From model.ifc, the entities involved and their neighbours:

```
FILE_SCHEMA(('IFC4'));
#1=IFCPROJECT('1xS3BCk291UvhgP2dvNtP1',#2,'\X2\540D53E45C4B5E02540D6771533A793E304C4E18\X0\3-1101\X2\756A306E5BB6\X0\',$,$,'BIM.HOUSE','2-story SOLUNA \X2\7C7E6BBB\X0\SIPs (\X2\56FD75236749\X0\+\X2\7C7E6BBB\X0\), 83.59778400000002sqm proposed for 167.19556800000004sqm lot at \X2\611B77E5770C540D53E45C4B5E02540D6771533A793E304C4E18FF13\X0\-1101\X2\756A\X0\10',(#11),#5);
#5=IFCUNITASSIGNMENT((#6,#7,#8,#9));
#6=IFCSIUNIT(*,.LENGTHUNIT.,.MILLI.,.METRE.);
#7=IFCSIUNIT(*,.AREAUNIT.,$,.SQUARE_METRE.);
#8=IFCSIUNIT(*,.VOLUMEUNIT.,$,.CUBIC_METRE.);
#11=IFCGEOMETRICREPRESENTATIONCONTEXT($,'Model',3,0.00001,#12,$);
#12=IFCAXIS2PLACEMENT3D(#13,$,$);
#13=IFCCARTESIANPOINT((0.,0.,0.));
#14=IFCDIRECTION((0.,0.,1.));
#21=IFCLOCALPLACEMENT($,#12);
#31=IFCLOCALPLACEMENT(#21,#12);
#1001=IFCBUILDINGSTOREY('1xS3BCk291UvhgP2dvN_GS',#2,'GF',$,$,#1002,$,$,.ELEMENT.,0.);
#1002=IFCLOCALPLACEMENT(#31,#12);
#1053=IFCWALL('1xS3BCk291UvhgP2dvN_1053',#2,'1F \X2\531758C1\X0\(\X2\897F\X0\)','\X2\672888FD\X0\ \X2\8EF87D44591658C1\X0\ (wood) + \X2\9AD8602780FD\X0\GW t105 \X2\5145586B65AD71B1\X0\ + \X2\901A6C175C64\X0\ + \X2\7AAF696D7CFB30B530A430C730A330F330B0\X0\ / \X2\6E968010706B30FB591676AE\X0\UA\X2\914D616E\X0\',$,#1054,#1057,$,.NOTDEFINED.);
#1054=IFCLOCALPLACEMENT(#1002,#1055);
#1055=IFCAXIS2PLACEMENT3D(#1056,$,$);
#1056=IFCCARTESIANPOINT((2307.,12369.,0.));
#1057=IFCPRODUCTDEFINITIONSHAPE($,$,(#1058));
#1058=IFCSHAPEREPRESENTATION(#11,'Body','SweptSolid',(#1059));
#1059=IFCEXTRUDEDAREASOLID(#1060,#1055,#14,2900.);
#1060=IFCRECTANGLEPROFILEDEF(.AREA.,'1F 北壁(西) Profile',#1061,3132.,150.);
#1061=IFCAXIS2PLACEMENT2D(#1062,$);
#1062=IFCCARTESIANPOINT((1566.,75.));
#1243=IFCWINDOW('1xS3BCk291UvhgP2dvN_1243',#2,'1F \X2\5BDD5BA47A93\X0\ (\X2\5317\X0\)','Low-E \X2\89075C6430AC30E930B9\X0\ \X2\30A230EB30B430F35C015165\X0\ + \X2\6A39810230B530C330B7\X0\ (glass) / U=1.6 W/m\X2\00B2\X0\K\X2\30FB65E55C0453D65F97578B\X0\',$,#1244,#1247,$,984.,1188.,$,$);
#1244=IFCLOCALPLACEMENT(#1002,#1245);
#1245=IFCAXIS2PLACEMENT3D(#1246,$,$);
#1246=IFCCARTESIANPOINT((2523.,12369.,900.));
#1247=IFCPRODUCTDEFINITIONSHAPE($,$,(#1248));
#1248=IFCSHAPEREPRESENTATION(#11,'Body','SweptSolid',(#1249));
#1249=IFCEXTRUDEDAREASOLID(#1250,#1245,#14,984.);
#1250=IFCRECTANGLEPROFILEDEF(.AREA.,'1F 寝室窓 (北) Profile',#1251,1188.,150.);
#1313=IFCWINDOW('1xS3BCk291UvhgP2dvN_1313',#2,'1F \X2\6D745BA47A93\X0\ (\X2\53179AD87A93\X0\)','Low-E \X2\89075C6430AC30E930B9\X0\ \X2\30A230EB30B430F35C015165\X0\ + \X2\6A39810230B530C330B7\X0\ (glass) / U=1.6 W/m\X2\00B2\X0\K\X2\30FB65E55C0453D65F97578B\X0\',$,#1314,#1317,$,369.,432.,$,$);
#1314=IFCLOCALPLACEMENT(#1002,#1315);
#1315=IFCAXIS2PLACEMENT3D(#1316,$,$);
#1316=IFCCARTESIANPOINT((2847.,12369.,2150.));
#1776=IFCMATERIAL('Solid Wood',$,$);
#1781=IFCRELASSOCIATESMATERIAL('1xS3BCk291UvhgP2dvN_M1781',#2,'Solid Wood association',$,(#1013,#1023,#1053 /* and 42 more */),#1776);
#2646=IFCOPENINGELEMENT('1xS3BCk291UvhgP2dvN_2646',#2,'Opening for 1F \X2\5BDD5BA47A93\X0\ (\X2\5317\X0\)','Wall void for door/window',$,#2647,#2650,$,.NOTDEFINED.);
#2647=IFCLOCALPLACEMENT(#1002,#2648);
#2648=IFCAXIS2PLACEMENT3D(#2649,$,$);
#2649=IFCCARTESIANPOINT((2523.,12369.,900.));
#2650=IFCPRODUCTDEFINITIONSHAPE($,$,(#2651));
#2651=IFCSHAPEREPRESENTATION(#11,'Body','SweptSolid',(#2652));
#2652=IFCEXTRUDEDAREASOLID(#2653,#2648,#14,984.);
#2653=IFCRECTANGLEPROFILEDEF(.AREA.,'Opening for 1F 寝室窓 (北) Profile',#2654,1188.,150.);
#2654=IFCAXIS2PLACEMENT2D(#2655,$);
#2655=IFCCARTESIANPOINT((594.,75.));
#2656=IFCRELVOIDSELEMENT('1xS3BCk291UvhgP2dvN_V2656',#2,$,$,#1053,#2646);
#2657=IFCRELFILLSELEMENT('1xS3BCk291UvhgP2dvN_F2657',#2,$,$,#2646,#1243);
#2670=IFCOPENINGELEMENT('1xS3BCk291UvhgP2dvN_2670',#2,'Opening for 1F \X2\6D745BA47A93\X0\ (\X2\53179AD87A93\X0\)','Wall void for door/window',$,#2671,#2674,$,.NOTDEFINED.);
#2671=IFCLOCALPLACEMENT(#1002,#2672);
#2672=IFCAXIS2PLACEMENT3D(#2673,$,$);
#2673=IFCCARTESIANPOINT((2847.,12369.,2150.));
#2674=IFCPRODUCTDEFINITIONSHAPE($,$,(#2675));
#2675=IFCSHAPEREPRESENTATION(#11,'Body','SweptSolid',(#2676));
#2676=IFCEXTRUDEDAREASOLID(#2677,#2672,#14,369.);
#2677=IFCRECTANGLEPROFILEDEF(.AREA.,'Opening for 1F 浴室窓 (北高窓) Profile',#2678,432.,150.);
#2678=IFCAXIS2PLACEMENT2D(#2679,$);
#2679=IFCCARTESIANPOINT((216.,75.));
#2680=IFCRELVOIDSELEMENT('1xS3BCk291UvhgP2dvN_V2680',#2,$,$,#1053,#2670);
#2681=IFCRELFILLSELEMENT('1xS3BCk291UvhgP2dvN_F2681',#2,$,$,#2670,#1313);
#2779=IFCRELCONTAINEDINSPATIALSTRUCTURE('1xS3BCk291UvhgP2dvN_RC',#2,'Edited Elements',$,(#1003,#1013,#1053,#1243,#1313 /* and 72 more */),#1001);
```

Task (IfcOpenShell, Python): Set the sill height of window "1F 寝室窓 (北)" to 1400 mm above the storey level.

```python
import numpy as np
import ifcopenshell
import ifcopenshell.api.geometry
import ifcopenshell.geom
import ifcopenshell.util.element
import ifcopenshell.util.placement
import ifcopenshell.util.shape
import ifcopenshell.util.unit

model = ifcopenshell.open("model.ifc")
unit_scale = ifcopenshell.util.unit.calculate_unit_scale(model)

window = model.by_guid("1xS3BCk291UvhgP2dvN_1243")
opening = window.FillsVoids[0].RelatingOpeningElement
storey = ifcopenshell.util.element.get_container(window, ifc_class="IfcBuildingStorey")
level = ifcopenshell.util.placement.get_local_placement(storey.ObjectPlacement)[2, 3]

# The opening's origin need not be at the sill, so measure its lowest point.
shape = ifcopenshell.geom.create_shape(ifcopenshell.geom.settings(), opening)
bottom = ifcopenshell.util.shape.get_shape_bottom_elevation(shape, shape.geometry) / unit_scale
dz = level + 1.4 / unit_scale - bottom

shift = np.array([0.0, 0.0, dz])
# The window is not placed relative to its opening, so move both.
for product in (opening, window):
    matrix = ifcopenshell.util.placement.get_local_placement(product.ObjectPlacement)
    matrix[:3, 3] += shift
    ifcopenshell.api.geometry.edit_object_placement(model, product=product, matrix=matrix, is_si=False)

print(f"moved by {dz * unit_scale:+.3f} m")

model.write("model_edited.ifc")
```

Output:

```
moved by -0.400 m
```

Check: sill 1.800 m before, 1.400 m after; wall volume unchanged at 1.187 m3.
